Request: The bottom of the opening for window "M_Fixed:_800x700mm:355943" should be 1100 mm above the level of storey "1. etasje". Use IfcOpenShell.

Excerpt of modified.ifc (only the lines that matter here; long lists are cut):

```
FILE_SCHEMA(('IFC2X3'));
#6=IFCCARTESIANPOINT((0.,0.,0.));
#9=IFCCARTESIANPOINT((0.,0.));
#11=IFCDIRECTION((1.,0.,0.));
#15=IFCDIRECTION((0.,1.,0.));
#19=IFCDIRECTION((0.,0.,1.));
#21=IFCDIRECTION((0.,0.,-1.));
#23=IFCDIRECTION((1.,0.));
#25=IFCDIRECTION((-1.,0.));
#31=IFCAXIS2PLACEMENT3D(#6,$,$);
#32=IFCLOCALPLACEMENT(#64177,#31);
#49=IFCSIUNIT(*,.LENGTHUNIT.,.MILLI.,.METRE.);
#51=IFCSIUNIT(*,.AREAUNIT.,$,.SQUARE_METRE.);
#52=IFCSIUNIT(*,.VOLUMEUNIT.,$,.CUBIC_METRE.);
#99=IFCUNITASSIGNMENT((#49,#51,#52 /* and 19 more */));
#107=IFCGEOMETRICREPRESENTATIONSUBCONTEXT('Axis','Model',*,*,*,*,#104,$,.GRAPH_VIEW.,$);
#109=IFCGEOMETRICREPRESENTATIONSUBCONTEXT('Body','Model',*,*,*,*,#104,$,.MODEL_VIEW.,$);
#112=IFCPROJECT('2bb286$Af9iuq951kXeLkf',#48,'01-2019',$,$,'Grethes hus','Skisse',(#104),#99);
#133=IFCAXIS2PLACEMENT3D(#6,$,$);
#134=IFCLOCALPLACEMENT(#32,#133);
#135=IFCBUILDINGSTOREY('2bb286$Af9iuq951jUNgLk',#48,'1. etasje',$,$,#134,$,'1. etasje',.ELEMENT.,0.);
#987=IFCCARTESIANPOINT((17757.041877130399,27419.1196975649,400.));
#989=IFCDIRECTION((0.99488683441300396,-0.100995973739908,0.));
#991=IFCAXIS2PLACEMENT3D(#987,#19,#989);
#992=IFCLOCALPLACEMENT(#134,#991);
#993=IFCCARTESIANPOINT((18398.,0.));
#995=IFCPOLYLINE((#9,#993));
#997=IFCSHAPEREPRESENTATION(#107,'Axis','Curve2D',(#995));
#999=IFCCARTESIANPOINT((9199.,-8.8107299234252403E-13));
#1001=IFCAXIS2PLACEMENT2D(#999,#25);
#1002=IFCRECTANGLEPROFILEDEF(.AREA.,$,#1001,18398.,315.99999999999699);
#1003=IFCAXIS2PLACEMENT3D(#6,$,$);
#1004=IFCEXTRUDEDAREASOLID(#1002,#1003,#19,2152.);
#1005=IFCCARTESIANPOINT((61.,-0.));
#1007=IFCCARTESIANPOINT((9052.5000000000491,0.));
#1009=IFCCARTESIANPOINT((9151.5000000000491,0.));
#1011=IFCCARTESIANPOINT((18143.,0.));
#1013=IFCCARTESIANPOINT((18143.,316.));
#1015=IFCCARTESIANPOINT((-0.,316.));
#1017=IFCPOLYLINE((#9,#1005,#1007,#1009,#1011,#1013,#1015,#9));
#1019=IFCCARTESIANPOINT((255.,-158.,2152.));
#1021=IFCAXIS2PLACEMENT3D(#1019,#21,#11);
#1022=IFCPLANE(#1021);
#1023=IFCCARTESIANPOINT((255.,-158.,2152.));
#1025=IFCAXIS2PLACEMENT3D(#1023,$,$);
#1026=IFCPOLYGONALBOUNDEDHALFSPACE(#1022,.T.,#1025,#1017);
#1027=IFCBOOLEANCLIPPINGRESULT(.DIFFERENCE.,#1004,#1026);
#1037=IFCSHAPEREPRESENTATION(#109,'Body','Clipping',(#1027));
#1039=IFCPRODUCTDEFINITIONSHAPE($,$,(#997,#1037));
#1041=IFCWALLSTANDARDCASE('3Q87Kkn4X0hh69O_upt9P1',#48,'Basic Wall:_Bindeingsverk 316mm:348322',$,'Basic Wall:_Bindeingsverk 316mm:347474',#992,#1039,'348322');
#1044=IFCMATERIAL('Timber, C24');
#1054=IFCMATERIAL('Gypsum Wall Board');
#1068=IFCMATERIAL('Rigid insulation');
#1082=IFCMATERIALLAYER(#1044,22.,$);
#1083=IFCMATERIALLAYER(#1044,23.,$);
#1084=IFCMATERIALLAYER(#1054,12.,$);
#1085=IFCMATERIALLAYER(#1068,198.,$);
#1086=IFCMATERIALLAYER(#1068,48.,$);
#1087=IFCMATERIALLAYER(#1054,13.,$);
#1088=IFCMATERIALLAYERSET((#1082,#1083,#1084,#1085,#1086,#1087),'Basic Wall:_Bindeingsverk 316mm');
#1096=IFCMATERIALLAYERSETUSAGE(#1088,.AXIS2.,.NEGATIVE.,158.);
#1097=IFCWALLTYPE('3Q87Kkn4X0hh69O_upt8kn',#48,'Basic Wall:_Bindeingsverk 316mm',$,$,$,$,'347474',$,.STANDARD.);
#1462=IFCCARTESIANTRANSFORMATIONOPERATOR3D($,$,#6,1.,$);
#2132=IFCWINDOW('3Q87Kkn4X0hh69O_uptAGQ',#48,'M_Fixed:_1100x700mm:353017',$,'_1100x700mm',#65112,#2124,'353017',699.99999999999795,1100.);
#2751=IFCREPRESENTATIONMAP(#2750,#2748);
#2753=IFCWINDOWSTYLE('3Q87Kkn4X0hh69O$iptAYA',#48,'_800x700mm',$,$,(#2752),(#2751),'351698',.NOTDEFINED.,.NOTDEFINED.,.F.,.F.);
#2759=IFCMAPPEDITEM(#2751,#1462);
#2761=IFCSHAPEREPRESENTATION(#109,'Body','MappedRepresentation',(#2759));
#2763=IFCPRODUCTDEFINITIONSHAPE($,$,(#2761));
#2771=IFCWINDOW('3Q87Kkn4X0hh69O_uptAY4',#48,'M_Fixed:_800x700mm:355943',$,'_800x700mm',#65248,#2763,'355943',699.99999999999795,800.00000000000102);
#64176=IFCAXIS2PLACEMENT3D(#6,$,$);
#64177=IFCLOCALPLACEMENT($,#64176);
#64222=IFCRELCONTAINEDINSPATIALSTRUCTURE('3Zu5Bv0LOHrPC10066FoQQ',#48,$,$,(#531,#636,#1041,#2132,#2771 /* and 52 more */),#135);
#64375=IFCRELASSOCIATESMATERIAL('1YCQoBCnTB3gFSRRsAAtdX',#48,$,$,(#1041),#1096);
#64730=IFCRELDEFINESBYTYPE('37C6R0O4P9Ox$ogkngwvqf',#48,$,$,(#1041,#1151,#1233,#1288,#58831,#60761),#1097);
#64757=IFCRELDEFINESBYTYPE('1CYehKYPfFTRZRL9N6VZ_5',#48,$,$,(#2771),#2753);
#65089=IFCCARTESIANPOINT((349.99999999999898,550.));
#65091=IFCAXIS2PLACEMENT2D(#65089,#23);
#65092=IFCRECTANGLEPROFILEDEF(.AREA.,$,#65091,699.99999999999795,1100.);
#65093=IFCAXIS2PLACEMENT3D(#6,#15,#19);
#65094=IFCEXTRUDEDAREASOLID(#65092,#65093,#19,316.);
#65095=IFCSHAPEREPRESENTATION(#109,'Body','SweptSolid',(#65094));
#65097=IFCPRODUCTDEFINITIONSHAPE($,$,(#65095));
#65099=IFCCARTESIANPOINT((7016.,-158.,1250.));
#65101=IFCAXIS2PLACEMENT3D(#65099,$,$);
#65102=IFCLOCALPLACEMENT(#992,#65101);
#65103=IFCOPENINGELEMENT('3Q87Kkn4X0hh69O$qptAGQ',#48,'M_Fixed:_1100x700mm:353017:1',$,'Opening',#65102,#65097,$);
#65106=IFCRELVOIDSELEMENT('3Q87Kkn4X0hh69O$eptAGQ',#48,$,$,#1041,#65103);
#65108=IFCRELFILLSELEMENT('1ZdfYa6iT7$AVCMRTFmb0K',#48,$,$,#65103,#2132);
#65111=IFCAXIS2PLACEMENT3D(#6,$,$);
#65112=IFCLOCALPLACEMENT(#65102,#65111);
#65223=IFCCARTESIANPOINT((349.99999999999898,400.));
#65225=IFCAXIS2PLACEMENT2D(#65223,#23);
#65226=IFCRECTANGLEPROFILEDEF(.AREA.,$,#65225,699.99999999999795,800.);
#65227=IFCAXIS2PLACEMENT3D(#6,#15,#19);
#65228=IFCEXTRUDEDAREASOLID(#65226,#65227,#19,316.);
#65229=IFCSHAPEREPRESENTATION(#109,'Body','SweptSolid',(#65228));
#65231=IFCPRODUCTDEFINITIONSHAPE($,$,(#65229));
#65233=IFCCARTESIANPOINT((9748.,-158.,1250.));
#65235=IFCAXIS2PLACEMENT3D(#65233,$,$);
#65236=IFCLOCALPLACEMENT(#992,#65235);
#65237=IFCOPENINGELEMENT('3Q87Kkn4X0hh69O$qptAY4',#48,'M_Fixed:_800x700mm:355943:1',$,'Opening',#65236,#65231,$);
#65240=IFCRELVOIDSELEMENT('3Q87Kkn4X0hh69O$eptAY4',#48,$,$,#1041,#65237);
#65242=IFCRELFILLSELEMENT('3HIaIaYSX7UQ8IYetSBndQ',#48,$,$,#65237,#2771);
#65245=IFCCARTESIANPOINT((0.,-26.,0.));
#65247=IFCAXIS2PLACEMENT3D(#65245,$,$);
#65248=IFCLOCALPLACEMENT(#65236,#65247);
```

```python
import numpy as np
import ifcopenshell
import ifcopenshell.api.geometry
import ifcopenshell.geom
import ifcopenshell.util.element
import ifcopenshell.util.placement
import ifcopenshell.util.shape
import ifcopenshell.util.unit

model = ifcopenshell.open("modified.ifc")
unit_scale = ifcopenshell.util.unit.calculate_unit_scale(model)

window = model.by_guid("3Q87Kkn4X0hh69O_uptAY4")
opening = window.FillsVoids[0].RelatingOpeningElement
storey = ifcopenshell.util.element.get_container(window, ifc_class="IfcBuildingStorey")
level = ifcopenshell.util.placement.get_local_placement(storey.ObjectPlacement)[2, 3]

# The opening's origin need not be at the sill, so measure its lowest point.
shape = ifcopenshell.geom.create_shape(ifcopenshell.geom.settings(), opening)
bottom = ifcopenshell.util.shape.get_shape_bottom_elevation(shape, shape.geometry) / unit_scale
dz = level + 1100.0 - bottom

shift = np.array([0.0, 0.0, dz])
# The window is placed relative to its opening, so it follows when the opening moves.
matrix = ifcopenshell.util.placement.get_local_placement(opening.ObjectPlacement)
matrix[:3, 3] += shift
ifcopenshell.api.geometry.edit_object_placement(
    model, product=opening, matrix=matrix, is_si=False, should_transform_children=True
)

print(f"moved by {dz * unit_scale:+.3f} m")

model.write("modified_v2.ifc")
```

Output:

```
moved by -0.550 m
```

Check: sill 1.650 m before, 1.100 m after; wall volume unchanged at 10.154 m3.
